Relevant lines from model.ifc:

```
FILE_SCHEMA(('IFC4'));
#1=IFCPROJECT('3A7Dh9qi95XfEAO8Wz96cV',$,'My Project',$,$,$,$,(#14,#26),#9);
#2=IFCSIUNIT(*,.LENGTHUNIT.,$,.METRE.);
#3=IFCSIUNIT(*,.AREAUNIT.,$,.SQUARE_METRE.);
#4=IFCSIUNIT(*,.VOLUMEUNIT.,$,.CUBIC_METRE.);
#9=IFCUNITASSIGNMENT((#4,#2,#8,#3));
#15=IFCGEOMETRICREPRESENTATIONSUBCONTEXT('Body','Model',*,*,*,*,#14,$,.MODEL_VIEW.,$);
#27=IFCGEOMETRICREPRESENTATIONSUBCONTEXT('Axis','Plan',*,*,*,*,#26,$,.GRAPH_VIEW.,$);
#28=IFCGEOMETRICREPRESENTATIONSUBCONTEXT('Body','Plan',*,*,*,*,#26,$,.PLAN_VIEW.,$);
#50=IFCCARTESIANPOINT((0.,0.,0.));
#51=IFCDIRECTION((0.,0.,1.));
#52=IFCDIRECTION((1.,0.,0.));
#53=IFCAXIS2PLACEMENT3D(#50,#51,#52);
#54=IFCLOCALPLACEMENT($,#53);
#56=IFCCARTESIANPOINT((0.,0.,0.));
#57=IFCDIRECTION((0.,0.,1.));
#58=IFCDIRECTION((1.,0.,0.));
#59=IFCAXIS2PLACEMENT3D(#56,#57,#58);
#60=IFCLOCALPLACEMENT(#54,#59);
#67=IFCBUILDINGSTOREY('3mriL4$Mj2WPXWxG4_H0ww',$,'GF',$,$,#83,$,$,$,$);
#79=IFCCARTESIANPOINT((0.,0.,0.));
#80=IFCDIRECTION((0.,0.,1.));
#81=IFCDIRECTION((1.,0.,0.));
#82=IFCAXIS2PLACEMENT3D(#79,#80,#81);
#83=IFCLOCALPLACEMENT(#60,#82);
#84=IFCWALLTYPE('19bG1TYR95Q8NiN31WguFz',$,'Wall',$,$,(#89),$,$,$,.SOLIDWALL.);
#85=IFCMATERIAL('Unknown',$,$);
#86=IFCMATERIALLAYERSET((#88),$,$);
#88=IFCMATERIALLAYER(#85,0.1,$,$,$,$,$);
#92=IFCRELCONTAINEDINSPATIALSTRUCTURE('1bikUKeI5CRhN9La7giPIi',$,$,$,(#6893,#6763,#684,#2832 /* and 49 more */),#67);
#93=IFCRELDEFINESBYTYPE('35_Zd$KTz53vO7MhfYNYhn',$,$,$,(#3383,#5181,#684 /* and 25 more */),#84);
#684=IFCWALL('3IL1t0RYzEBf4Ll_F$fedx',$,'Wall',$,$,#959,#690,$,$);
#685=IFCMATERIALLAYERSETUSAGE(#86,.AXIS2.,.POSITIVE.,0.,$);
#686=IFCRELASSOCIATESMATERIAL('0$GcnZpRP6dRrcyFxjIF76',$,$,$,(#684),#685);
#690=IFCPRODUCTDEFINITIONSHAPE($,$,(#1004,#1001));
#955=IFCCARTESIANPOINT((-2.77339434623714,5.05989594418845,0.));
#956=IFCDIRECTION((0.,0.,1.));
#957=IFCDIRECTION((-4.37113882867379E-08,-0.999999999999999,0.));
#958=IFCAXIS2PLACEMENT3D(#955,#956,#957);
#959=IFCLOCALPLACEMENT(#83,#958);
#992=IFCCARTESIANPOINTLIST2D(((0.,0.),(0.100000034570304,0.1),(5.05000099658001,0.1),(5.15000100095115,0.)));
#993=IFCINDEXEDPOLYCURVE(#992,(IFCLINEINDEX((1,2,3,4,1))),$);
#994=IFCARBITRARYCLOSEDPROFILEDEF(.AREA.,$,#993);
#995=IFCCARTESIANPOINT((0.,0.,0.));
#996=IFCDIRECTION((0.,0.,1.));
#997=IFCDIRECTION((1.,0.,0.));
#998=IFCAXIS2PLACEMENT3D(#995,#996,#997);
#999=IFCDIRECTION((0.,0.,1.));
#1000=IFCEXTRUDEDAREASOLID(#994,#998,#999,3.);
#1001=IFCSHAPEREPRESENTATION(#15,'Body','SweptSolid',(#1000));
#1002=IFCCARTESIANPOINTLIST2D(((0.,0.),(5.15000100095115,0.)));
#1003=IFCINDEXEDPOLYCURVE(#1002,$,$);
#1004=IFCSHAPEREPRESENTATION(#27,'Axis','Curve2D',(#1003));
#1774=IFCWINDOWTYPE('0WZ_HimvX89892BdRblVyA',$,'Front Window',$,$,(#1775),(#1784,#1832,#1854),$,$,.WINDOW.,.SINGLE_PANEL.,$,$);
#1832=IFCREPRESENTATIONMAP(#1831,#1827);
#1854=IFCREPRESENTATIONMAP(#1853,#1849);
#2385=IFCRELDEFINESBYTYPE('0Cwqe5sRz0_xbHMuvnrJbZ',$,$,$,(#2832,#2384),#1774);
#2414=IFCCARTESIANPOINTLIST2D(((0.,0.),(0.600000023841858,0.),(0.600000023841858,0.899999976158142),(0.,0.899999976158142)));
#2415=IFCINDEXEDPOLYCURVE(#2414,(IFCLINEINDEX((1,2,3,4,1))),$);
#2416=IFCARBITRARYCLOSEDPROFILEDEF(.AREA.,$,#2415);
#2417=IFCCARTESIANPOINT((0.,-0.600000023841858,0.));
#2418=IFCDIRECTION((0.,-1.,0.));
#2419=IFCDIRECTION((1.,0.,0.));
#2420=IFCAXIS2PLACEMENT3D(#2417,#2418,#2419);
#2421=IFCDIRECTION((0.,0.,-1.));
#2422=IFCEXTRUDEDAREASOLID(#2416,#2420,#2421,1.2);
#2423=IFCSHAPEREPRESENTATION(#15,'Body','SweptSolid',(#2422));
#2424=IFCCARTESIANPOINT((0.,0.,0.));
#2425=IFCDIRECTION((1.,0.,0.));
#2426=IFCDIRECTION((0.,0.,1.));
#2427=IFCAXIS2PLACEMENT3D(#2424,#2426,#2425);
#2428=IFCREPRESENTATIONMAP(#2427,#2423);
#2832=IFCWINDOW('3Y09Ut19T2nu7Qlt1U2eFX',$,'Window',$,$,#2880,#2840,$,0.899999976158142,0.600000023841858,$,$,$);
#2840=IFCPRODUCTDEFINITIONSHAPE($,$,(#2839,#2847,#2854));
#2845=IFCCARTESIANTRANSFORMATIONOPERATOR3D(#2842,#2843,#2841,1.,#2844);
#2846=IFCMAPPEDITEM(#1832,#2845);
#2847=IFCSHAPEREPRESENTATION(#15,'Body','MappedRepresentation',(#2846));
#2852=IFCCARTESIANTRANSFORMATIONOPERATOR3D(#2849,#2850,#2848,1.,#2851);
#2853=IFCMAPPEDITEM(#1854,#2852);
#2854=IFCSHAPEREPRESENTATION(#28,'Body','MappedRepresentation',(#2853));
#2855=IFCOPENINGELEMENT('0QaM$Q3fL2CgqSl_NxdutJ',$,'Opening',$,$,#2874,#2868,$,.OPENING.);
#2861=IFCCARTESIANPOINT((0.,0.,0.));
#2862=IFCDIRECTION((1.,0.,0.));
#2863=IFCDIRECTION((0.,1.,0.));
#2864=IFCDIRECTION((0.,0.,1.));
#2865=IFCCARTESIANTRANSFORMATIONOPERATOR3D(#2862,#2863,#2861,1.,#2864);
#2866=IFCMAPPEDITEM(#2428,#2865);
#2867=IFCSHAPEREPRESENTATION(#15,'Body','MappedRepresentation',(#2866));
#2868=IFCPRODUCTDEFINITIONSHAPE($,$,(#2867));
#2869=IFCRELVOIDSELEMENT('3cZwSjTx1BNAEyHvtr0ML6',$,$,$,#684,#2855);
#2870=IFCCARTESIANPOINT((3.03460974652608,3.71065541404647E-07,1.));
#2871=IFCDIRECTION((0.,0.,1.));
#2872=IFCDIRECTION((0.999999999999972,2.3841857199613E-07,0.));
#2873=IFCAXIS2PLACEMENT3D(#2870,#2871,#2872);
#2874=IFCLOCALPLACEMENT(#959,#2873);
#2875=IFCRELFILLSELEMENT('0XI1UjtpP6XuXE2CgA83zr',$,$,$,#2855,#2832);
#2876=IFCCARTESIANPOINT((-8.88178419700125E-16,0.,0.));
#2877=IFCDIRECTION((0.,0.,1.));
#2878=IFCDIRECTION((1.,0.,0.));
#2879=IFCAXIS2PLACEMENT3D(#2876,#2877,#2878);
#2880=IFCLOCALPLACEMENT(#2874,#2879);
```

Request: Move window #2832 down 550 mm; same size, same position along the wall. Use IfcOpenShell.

```python
import numpy as np
import ifcopenshell
import ifcopenshell.api.geometry
import ifcopenshell.util.placement
import ifcopenshell.util.unit

model = ifcopenshell.open("model.ifc")
unit_scale = ifcopenshell.util.unit.calculate_unit_scale(model)

window = model.by_guid("3Y09Ut19T2nu7Qlt1U2eFX")
opening = window.FillsVoids[0].RelatingOpeningElement
dz = -0.55

shift = np.array([0.0, 0.0, dz])
# The window is placed relative to its opening, so it follows when the opening moves.
matrix = ifcopenshell.util.placement.get_local_placement(opening.ObjectPlacement)
matrix[:3, 3] += shift
ifcopenshell.api.geometry.edit_object_placement(
    model, product=opening, matrix=matrix, is_si=False, should_transform_children=True
)

print(f"moved by {dz * unit_scale:+.3f} m")

model.write("model_rev.ifc")
```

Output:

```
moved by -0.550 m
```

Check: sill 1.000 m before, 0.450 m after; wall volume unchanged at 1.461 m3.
